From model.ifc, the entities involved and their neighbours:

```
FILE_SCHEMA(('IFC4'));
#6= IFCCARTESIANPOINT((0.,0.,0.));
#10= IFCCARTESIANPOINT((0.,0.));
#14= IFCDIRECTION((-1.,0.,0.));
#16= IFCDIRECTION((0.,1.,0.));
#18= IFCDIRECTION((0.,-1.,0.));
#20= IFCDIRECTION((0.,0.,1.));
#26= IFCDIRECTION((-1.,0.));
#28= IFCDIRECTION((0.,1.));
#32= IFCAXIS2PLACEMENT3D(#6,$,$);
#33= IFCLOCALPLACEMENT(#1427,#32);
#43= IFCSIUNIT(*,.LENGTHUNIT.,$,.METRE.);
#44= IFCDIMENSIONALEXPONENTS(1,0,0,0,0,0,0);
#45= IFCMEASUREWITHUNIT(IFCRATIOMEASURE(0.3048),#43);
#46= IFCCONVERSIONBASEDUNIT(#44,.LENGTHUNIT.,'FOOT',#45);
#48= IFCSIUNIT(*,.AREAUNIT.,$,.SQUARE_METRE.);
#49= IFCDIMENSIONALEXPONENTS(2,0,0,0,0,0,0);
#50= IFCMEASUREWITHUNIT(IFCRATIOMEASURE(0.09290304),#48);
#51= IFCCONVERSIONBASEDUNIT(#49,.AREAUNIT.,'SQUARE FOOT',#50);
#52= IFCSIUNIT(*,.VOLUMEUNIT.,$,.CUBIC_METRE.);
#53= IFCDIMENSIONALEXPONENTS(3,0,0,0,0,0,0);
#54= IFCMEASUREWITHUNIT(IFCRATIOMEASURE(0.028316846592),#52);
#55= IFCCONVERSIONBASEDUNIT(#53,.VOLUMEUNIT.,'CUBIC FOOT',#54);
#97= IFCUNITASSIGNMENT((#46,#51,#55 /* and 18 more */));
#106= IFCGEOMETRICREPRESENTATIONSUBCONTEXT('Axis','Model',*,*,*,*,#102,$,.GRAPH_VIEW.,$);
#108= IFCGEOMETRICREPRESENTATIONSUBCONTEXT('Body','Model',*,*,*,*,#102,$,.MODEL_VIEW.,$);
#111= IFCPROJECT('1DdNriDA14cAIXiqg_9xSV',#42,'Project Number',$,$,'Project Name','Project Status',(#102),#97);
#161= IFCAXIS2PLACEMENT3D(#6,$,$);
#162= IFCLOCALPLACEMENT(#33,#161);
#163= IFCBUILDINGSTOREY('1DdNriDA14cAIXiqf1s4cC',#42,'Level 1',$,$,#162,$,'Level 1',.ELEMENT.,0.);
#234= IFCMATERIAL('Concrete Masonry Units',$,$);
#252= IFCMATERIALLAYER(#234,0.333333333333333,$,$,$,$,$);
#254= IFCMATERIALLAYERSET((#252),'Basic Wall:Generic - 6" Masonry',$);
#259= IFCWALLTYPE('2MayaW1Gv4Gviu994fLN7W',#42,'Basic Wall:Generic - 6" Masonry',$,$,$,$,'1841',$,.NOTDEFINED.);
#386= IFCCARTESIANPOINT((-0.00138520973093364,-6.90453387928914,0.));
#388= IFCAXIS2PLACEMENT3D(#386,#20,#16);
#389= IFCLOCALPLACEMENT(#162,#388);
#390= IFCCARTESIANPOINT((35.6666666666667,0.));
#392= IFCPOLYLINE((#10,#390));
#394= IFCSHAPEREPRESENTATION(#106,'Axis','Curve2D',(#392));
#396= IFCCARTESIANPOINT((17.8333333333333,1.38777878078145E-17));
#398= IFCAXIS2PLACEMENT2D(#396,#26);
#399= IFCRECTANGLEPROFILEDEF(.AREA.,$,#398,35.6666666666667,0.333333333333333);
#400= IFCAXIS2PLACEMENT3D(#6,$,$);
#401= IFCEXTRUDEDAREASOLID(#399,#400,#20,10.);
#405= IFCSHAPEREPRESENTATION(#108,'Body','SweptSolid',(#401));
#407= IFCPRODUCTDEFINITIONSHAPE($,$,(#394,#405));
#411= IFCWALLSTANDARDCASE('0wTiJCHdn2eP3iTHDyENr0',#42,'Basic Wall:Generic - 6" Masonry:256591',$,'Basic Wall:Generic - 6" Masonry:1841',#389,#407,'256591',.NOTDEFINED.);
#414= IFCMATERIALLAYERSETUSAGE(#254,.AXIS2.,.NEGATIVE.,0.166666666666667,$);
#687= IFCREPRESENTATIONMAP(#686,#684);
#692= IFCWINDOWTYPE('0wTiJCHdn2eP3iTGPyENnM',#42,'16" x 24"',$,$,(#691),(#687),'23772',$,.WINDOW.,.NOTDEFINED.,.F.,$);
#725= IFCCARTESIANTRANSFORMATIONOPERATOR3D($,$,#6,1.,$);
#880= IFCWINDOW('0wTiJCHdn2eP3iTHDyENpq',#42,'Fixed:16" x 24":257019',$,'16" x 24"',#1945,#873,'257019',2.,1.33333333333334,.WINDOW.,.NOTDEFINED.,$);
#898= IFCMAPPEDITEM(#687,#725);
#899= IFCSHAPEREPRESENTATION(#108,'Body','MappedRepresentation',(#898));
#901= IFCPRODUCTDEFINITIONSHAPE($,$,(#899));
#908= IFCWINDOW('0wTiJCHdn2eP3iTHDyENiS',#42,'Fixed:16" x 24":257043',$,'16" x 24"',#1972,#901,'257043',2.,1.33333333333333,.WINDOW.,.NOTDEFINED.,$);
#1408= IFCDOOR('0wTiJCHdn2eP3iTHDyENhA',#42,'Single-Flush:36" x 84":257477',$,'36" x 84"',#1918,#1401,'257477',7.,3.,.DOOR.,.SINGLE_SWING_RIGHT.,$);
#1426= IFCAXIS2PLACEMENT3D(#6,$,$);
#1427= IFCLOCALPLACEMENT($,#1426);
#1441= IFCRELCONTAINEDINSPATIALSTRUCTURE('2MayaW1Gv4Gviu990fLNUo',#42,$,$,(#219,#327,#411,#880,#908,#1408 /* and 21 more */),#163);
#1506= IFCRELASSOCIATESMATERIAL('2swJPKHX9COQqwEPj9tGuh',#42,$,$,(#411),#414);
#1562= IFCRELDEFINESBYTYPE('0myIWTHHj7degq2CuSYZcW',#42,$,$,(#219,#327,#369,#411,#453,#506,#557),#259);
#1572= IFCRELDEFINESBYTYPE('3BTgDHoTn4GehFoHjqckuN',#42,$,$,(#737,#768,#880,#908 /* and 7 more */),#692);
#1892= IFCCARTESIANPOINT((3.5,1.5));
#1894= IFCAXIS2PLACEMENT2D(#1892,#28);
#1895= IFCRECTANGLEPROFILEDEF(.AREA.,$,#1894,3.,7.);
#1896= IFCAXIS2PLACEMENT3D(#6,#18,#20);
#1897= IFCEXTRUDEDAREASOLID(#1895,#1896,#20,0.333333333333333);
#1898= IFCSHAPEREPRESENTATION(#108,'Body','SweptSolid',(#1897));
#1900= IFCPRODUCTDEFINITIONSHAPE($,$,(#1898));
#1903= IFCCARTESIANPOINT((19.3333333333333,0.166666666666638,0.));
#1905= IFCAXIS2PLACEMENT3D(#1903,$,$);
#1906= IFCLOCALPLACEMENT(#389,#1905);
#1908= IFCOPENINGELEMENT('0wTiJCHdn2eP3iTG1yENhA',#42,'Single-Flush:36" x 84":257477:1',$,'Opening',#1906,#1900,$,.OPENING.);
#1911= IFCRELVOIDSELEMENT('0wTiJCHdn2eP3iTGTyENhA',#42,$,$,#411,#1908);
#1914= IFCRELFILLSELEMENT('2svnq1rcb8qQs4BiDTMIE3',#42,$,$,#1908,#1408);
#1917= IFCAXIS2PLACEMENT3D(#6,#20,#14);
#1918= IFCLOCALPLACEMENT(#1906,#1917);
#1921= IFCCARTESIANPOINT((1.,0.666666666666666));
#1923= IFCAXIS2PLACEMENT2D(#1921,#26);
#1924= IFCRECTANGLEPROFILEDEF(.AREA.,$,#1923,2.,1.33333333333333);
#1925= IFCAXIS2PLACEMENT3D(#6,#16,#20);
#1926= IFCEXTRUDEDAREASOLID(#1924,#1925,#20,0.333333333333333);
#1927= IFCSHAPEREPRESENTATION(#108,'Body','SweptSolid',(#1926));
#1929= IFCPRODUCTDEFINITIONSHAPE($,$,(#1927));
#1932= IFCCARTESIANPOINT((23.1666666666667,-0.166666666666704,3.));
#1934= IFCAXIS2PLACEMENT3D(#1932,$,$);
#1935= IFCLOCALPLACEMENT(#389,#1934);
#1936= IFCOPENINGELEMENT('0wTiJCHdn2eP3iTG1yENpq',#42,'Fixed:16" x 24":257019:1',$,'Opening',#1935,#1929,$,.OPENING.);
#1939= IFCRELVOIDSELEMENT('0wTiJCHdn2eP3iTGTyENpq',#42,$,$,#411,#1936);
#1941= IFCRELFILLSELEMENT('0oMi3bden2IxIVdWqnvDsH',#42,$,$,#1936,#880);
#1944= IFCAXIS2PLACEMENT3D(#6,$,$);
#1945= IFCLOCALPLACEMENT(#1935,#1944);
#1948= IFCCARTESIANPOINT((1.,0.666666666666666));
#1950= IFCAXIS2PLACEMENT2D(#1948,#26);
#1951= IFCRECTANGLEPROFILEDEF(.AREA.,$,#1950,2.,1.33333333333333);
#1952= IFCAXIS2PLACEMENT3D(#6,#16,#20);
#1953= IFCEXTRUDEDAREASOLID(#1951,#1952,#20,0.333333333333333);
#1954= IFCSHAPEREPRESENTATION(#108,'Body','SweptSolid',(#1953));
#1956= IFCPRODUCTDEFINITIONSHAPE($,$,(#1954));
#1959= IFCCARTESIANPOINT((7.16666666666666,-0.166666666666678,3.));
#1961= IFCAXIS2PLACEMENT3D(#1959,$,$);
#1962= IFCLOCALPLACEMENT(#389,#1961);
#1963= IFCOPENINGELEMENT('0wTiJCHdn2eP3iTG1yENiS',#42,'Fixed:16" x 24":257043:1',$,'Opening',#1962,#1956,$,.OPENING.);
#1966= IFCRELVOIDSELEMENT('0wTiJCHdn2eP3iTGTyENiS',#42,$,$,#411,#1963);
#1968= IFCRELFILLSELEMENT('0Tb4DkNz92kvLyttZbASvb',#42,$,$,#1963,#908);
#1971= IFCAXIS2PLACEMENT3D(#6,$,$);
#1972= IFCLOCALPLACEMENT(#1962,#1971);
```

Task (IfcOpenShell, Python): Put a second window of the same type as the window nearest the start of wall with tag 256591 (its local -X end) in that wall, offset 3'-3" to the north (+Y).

```python
import ifcopenshell
import ifcopenshell.api.feature
import ifcopenshell.api.geometry
import ifcopenshell.api.root
import ifcopenshell.geom
import ifcopenshell.util.element
import ifcopenshell.util.placement
import ifcopenshell.util.shape
import ifcopenshell.util.unit

model = ifcopenshell.open("model.ifc")
unit_scale = ifcopenshell.util.unit.calculate_unit_scale(model)
settings = ifcopenshell.geom.settings()


def volume(element):
    """Net volume in cubic metres, openings subtracted."""
    shape = ifcopenshell.geom.create_shape(settings, element)
    return ifcopenshell.util.shape.get_volume(shape.geometry)


def reuse_history(source, copy):
    """copy_class also copies each property set's owner history, people and application; keep the originals."""
    for rel in copy.IsDefinedBy:
        if rel.is_a("IfcRelDefinesByProperties") and (history := rel.RelatingPropertyDefinition.OwnerHistory):
            rel.RelatingPropertyDefinition.OwnerHistory = source.OwnerHistory
            ifcopenshell.util.element.remove_deep2(model, history)


window = model.by_id(908)
opening = window.FillsVoids[0].RelatingOpeningElement
wall = opening.VoidsElements[0].RelatingBuildingElement
before = volume(wall)
shift = ifcopenshell.util.placement.get_local_placement(wall.ObjectPlacement)[:3, 0] * 39 * 0.0254 / unit_scale

# copy_class copies the void relationship, type, container and properties, but no geometry.
new_opening = ifcopenshell.api.root.copy_class(model, product=opening)
new_opening.Representation = ifcopenshell.util.element.copy_deep(
    model, opening.Representation, exclude=["IfcGeometricRepresentationContext", "IfcRepresentationMap"]
)
new_opening.Name = 'Fixed:16" x 24"'
new_window = ifcopenshell.api.root.copy_class(model, product=window)
new_window.Representation = ifcopenshell.util.element.copy_deep(
    model, window.Representation, exclude=["IfcGeometricRepresentationContext", "IfcRepresentationMap"]
)
new_window.Name = 'Fixed:16" x 24"'
new_window.Tag = None
reuse_history(window, new_window)
ifcopenshell.api.feature.add_filling(model, opening=new_opening, element=new_window)

for old, new in ((opening, new_opening), (window, new_window)):
    matrix = ifcopenshell.util.placement.get_local_placement(old.ObjectPlacement)
    matrix[:3, 3] += shift
    ifcopenshell.api.geometry.edit_object_placement(model, product=new, matrix=matrix, is_si=False)

after = volume(wall)

print(f"wall volume {before:.3f} -> {after:.3f} m3")

model.write("model_edited.ifc")
```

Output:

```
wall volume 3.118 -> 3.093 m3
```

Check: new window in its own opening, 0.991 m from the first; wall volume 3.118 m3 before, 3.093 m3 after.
